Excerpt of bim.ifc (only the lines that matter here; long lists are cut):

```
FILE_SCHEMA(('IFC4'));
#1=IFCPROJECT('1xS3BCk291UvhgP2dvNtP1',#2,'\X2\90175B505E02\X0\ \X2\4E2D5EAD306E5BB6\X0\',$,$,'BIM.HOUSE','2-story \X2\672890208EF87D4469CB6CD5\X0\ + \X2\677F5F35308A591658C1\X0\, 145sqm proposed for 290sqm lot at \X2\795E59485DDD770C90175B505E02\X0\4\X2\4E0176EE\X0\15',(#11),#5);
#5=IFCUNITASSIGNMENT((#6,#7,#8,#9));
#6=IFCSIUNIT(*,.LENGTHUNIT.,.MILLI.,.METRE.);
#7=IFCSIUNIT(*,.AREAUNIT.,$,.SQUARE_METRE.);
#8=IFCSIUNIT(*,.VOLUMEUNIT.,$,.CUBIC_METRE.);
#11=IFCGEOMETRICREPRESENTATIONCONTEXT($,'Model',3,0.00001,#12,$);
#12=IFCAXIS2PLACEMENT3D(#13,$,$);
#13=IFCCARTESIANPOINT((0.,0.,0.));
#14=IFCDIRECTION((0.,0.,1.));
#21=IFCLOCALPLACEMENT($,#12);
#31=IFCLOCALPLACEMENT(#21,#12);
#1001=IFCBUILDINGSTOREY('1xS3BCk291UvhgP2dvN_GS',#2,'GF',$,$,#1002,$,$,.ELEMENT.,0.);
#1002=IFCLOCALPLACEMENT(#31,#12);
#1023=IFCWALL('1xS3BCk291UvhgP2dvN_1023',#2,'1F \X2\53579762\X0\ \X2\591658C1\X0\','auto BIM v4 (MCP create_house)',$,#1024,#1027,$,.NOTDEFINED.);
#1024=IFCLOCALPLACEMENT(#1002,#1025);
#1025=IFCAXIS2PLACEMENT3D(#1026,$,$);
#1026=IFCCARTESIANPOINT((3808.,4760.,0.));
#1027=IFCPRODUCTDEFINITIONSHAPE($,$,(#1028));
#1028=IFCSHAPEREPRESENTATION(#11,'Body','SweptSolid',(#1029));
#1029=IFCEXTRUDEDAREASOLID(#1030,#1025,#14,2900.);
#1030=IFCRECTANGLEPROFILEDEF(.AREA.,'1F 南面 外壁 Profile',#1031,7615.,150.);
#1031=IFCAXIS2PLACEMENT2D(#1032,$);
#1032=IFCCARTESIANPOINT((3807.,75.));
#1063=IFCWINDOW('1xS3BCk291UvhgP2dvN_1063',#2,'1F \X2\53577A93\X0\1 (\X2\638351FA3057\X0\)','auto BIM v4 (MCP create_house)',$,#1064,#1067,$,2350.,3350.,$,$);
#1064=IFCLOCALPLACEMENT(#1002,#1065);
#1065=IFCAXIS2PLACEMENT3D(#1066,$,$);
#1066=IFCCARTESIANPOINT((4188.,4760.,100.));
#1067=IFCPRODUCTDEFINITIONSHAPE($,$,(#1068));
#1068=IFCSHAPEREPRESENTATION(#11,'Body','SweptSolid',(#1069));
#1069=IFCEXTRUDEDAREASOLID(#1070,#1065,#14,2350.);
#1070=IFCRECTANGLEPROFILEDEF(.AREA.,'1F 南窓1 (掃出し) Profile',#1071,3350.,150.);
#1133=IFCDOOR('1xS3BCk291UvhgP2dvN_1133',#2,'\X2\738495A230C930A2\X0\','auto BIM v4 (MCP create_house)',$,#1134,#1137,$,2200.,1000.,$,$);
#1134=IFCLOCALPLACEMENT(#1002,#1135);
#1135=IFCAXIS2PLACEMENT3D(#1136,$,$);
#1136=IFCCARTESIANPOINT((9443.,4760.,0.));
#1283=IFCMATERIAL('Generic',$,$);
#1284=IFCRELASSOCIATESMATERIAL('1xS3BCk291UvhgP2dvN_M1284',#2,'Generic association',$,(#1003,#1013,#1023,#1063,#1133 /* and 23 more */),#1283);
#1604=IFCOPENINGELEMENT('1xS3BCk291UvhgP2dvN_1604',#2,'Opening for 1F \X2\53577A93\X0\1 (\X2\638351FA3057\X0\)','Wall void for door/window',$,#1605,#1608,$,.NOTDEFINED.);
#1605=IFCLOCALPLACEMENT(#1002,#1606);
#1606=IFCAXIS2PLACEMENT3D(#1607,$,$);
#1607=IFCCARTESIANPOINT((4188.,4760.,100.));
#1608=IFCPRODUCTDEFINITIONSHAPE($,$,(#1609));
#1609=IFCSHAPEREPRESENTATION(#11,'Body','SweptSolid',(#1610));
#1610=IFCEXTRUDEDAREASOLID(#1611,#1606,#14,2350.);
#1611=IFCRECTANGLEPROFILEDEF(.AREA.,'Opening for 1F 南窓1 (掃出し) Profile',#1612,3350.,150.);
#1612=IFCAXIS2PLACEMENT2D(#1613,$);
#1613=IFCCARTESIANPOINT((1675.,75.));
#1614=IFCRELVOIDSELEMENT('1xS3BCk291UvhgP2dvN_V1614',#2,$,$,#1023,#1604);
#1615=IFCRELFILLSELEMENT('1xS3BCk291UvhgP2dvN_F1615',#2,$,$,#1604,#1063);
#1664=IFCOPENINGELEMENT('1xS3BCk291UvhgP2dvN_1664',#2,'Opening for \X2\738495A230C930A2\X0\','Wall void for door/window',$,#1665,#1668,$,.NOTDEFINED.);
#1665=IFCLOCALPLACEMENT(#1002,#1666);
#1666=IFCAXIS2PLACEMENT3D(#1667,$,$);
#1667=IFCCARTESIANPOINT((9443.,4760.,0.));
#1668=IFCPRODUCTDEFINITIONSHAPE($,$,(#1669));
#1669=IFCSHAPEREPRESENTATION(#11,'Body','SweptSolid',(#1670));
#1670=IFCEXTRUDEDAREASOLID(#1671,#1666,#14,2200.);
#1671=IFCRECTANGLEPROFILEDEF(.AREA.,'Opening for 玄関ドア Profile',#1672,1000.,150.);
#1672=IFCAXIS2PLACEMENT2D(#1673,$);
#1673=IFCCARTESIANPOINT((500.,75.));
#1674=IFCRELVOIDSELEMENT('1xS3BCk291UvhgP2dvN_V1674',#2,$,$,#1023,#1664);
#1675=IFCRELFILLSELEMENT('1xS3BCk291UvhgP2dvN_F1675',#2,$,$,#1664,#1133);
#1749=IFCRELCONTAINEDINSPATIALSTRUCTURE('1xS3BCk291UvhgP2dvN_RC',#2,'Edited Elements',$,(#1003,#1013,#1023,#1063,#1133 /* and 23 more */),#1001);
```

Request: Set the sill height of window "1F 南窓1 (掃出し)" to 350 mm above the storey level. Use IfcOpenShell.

```python
import numpy as np
import ifcopenshell
import ifcopenshell.api.geometry
import ifcopenshell.geom
import ifcopenshell.util.element
import ifcopenshell.util.placement
import ifcopenshell.util.shape
import ifcopenshell.util.unit

model = ifcopenshell.open("bim.ifc")
unit_scale = ifcopenshell.util.unit.calculate_unit_scale(model)

window = model.by_guid("1xS3BCk291UvhgP2dvN_1063")
opening = window.FillsVoids[0].RelatingOpeningElement
storey = ifcopenshell.util.element.get_container(window, ifc_class="IfcBuildingStorey")
level = ifcopenshell.util.placement.get_local_placement(storey.ObjectPlacement)[2, 3]

# The opening's origin need not be at the sill, so measure its lowest point.
shape = ifcopenshell.geom.create_shape(ifcopenshell.geom.settings(), opening)
bottom = ifcopenshell.util.shape.get_shape_bottom_elevation(shape, shape.geometry) / unit_scale
dz = level + 0.35 / unit_scale - bottom

shift = np.array([0.0, 0.0, dz])
# The window is not placed relative to its opening, so move both.
for product in (opening, window):
    matrix = ifcopenshell.util.placement.get_local_placement(product.ObjectPlacement)
    matrix[:3, 3] += shift
    ifcopenshell.api.geometry.edit_object_placement(model, product=product, matrix=matrix, is_si=False)

print(f"moved by {dz * unit_scale:+.3f} m")

model.write("bim_updated.ifc")
```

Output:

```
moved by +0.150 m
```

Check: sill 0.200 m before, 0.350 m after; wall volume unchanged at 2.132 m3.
